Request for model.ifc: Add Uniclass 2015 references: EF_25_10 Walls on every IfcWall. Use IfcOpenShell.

First a look at what the model holds.

```python
import ifcopenshell

model = ifcopenshell.open("model.ifc")
print(model.schema)
print("classifications:", [c.Name for c in model.by_type("IfcClassification")])
for ifc_class in ("IfcDoor", "IfcRoof", "IfcStair", "IfcWall", "IfcWindow"):
    print(ifc_class, len(model.by_type(ifc_class)))
```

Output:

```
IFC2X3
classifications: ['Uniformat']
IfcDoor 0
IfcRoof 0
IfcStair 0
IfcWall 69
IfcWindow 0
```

```python
import ifcopenshell
import ifcopenshell.api.classification

model = ifcopenshell.open("model.ifc")

# IFC2X3 requires Source and Edition and has no link from the project to the system.
system = model.create_entity("IfcClassification", Source="NBS", Edition="2015", Name="Uniclass 2015")

codes = {
    "IfcWall": ("EF_25_10", "Walls"),
}
for ifc_class, (code, name) in codes.items():
    products = model.by_type(ifc_class)
    ifcopenshell.api.classification.add_reference(
        model, products=products, classification=system, identification=code, name=name
    )
    print(code, len(products))

model.write("model_updated.ifc")
```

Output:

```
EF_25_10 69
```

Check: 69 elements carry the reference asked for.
